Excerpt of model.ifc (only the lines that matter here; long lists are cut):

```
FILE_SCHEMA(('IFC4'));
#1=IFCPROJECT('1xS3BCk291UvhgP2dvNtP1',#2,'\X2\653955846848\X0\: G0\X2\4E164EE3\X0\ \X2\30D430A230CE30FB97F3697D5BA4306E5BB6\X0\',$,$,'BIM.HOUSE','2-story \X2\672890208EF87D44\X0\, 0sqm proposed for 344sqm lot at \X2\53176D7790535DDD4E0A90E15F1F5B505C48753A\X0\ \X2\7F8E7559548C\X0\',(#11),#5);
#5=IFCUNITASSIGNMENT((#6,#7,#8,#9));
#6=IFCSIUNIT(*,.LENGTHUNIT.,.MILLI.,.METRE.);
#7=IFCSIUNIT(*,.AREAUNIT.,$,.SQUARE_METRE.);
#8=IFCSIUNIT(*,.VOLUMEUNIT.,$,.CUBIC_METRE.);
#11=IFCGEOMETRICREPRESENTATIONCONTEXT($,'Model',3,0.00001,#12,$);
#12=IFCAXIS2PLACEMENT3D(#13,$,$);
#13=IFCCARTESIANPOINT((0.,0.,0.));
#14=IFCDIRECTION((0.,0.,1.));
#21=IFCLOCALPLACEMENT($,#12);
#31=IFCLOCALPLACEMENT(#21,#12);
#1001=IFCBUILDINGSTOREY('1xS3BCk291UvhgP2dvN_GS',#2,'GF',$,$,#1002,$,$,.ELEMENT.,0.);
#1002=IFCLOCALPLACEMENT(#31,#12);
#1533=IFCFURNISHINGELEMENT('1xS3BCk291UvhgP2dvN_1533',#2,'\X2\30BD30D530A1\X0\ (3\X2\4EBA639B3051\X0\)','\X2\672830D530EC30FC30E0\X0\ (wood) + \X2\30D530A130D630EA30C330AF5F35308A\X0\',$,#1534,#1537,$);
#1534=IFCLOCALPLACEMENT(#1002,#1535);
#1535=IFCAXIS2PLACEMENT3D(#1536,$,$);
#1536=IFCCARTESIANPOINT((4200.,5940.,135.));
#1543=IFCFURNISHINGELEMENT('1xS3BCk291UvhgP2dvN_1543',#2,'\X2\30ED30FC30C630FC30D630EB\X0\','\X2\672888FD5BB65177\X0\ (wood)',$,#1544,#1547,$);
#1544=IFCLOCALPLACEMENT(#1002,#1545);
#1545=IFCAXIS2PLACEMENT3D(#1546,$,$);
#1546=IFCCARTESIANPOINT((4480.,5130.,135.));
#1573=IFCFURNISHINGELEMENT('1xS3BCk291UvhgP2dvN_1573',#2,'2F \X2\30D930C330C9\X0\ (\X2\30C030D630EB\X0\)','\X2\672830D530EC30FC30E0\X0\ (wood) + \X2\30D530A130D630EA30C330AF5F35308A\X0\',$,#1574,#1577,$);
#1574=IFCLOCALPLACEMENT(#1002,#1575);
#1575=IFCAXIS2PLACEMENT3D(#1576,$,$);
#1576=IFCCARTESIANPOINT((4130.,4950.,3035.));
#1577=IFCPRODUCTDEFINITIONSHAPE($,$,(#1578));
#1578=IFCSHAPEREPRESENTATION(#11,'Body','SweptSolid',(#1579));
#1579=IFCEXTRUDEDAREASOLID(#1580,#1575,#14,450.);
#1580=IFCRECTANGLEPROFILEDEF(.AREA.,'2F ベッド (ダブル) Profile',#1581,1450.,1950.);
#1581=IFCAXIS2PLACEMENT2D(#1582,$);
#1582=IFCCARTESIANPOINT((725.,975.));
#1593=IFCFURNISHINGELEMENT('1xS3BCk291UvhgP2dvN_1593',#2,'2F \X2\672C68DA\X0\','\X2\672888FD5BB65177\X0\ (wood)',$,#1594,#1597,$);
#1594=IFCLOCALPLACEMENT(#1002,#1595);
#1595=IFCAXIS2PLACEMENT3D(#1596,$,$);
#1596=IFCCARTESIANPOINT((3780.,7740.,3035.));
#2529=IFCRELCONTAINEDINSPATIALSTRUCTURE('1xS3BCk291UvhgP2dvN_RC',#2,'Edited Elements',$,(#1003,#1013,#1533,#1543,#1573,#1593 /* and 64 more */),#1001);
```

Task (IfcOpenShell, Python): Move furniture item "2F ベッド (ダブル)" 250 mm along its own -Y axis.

```python
import ifcopenshell
import ifcopenshell.api.geometry
import ifcopenshell.util.placement
import ifcopenshell.util.unit

model = ifcopenshell.open("model.ifc")
unit_scale = ifcopenshell.util.unit.calculate_unit_scale(model)

item = model.by_guid("1xS3BCk291UvhgP2dvN_1573")
matrix = ifcopenshell.util.placement.get_local_placement(item.ObjectPlacement)
matrix[:3, 3] -= matrix[:3, 1] * 0.25 / unit_scale
ifcopenshell.api.geometry.edit_object_placement(model, product=item, matrix=matrix, is_si=False)

print(ifcopenshell.util.placement.get_local_placement(item.ObjectPlacement).round(3) + 0.0)

model.write("model-out.ifc")
```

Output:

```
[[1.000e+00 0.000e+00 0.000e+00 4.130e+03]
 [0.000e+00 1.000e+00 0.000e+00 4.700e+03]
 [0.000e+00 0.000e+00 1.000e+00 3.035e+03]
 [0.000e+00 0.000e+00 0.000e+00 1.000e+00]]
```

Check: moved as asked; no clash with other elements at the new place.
